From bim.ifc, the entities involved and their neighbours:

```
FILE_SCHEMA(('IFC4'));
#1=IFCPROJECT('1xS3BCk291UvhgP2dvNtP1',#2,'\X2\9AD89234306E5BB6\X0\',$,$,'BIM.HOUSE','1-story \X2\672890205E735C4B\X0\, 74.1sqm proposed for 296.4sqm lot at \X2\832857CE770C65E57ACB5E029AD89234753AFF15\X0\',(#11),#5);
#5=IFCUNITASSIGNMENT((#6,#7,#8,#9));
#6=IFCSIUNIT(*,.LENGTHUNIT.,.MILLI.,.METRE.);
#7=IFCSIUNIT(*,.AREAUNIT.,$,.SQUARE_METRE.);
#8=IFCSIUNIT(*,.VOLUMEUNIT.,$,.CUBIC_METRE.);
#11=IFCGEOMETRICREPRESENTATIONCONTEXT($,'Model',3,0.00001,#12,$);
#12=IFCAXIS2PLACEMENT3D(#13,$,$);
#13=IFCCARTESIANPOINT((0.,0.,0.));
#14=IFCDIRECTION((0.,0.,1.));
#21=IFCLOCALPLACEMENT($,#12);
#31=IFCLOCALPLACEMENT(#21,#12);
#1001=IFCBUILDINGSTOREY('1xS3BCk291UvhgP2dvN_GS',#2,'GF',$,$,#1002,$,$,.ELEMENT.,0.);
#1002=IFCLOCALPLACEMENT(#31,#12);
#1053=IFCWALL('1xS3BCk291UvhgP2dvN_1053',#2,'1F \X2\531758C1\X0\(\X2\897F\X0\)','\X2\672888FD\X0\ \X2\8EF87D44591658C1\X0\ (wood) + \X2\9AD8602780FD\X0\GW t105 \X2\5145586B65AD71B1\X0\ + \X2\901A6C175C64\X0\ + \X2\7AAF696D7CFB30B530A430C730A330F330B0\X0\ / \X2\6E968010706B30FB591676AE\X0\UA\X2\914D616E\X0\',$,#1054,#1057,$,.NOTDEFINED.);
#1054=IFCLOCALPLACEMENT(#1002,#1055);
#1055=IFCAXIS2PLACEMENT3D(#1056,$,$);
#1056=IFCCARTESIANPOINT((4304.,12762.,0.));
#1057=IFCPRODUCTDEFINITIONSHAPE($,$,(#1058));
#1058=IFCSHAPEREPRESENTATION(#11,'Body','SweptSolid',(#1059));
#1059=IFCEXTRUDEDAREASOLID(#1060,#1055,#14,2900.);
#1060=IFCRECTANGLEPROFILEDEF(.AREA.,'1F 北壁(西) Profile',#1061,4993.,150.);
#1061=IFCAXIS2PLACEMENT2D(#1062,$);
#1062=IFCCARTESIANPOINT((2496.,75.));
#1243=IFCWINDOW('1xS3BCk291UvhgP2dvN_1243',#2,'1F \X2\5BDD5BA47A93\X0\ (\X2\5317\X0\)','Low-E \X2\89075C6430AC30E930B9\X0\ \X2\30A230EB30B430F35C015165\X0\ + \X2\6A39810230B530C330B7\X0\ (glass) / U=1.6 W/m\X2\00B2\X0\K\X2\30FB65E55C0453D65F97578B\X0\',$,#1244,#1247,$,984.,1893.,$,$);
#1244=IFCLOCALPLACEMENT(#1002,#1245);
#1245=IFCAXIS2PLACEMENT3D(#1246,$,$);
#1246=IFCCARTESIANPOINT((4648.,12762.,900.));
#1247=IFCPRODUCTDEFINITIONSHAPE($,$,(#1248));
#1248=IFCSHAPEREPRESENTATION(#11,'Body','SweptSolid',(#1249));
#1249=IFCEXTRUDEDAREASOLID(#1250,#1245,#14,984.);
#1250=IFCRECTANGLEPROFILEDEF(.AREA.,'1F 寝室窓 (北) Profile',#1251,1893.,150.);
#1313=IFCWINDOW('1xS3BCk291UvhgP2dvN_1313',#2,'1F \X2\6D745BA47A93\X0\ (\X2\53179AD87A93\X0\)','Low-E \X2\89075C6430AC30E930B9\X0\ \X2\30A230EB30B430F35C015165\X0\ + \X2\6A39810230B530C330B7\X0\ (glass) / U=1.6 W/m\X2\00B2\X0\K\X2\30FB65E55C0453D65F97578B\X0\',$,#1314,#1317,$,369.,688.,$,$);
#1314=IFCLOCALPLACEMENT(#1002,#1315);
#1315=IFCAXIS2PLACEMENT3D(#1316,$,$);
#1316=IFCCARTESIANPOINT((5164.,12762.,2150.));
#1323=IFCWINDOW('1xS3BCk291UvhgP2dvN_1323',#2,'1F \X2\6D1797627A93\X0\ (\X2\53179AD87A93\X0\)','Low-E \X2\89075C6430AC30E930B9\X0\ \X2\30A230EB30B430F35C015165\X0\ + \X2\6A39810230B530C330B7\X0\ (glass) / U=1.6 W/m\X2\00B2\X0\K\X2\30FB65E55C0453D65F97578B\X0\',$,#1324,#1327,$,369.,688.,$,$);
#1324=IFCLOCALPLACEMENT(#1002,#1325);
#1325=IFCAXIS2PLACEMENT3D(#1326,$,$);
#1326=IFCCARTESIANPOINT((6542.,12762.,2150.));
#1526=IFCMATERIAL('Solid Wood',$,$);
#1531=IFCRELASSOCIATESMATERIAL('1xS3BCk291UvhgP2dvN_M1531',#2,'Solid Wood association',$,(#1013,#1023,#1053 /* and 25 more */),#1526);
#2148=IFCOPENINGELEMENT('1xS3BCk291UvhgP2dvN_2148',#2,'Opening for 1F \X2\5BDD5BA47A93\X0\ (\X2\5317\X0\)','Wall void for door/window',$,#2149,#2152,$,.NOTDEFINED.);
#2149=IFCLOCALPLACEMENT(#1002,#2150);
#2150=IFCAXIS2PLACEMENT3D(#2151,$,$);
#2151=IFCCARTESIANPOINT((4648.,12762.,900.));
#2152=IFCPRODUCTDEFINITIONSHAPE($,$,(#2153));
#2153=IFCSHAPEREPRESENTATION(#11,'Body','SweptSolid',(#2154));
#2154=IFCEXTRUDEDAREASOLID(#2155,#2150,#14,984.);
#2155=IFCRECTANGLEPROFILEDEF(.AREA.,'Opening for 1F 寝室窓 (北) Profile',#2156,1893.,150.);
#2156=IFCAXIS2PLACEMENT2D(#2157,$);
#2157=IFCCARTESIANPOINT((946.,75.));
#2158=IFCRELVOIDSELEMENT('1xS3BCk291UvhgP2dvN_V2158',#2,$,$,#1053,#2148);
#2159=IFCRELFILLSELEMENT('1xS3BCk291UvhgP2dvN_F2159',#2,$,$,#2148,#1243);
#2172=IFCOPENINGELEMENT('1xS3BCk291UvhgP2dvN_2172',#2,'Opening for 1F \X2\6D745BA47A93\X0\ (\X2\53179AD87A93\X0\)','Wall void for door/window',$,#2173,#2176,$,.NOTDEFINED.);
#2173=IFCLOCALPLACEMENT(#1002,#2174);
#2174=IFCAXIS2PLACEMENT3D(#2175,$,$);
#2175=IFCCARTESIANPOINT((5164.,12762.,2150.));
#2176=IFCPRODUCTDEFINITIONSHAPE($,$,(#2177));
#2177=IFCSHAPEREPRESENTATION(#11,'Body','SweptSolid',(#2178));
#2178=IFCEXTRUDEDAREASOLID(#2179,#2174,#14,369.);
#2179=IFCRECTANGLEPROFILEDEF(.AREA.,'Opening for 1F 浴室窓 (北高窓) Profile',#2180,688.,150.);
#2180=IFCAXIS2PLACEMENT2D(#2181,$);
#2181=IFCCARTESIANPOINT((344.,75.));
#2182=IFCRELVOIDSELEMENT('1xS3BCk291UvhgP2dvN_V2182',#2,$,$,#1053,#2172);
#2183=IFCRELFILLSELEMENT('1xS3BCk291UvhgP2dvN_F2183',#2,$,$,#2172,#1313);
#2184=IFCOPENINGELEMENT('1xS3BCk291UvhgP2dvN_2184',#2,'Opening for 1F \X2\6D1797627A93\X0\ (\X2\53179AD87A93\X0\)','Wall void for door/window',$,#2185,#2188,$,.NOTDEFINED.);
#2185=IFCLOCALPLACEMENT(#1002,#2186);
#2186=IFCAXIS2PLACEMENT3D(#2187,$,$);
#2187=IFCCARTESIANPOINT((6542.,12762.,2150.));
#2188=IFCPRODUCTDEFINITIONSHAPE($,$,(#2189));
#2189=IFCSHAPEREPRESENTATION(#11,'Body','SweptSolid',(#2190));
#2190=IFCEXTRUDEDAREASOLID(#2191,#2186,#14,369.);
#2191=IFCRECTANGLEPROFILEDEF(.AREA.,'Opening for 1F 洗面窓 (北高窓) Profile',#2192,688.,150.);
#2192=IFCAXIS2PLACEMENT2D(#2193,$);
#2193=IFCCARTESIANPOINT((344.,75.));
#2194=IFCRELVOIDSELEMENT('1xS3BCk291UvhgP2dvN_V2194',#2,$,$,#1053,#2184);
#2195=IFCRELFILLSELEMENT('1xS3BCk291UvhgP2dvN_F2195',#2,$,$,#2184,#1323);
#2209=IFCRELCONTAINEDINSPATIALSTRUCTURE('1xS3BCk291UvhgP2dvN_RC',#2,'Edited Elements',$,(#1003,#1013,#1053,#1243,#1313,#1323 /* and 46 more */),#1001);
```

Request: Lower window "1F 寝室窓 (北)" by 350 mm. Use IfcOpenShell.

```python
import numpy as np
import ifcopenshell
import ifcopenshell.api.geometry
import ifcopenshell.util.placement
import ifcopenshell.util.unit

model = ifcopenshell.open("bim.ifc")
unit_scale = ifcopenshell.util.unit.calculate_unit_scale(model)

window = model.by_guid("1xS3BCk291UvhgP2dvN_1243")
opening = window.FillsVoids[0].RelatingOpeningElement
dz = -0.35 / unit_scale

shift = np.array([0.0, 0.0, dz])
# The window is not placed relative to its opening, so move both.
for product in (opening, window):
    matrix = ifcopenshell.util.placement.get_local_placement(product.ObjectPlacement)
    matrix[:3, 3] += shift
    ifcopenshell.api.geometry.edit_object_placement(model, product=product, matrix=matrix, is_si=False)

print(f"moved by {dz * unit_scale:+.3f} m")

model.write("bim-out.ifc")
```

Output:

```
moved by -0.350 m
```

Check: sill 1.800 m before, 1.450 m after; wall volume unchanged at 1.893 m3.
